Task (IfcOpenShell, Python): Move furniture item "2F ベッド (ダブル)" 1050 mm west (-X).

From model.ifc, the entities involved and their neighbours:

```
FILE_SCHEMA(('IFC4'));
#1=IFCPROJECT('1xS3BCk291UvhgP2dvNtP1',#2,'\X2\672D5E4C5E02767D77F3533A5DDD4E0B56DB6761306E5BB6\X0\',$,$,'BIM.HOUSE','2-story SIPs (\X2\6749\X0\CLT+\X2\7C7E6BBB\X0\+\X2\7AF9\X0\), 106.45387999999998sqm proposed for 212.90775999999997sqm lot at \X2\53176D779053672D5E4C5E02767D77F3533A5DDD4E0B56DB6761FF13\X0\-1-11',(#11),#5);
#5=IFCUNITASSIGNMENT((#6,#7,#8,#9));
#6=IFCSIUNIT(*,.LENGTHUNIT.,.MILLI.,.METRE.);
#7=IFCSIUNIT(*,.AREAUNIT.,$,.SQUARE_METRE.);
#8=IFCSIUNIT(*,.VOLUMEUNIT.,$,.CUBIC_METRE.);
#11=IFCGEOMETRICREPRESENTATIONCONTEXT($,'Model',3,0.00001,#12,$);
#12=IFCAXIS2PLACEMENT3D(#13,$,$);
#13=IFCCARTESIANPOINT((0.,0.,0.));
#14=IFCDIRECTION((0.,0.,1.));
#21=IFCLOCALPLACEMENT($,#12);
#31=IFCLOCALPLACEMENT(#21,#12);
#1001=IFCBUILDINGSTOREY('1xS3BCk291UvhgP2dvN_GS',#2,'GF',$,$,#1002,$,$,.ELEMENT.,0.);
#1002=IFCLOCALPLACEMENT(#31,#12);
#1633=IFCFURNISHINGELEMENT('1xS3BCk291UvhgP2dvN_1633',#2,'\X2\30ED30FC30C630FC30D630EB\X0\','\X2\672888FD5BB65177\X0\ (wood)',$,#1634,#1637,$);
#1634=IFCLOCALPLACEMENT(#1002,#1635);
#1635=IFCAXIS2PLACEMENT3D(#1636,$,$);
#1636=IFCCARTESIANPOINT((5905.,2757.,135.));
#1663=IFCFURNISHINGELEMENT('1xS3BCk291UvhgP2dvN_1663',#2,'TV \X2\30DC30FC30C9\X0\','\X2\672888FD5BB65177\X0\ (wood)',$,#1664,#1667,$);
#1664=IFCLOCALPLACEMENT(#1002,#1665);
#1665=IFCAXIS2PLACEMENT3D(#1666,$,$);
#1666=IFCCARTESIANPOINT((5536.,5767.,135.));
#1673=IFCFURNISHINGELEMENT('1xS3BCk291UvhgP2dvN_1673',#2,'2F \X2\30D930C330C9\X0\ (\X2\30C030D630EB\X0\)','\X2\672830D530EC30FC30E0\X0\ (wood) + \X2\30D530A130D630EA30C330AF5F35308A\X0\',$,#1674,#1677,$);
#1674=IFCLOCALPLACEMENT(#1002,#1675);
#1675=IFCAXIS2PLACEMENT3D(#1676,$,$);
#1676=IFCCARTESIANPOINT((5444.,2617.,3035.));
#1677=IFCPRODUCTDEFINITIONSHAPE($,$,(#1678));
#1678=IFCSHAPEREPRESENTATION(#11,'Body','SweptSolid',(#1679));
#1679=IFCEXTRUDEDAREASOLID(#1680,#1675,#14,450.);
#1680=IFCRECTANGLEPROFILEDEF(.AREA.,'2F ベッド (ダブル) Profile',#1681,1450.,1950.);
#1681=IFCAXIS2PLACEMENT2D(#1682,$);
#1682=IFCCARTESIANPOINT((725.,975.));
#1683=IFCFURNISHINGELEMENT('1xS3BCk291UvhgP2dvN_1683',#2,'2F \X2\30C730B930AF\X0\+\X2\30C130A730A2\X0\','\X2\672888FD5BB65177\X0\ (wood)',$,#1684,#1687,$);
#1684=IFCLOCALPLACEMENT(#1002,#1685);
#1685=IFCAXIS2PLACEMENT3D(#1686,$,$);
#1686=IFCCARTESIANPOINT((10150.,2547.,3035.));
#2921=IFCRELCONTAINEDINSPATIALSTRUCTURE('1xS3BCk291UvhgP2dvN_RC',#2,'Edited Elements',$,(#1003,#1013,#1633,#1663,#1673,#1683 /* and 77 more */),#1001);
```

```python
import ifcopenshell
import ifcopenshell.api.geometry
import ifcopenshell.util.placement

model = ifcopenshell.open("model.ifc")

item = model.by_guid("1xS3BCk291UvhgP2dvN_1673")
matrix = ifcopenshell.util.placement.get_local_placement(item.ObjectPlacement)
matrix[0, 3] -= 1050.0
ifcopenshell.api.geometry.edit_object_placement(model, product=item, matrix=matrix, is_si=False)

print(ifcopenshell.util.placement.get_local_placement(item.ObjectPlacement).round(3) + 0.0)

model.write("model_v2.ifc")
```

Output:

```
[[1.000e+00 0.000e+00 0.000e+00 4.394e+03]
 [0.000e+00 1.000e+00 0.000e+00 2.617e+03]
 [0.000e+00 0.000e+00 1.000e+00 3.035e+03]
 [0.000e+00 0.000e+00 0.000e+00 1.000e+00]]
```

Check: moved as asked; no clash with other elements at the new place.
